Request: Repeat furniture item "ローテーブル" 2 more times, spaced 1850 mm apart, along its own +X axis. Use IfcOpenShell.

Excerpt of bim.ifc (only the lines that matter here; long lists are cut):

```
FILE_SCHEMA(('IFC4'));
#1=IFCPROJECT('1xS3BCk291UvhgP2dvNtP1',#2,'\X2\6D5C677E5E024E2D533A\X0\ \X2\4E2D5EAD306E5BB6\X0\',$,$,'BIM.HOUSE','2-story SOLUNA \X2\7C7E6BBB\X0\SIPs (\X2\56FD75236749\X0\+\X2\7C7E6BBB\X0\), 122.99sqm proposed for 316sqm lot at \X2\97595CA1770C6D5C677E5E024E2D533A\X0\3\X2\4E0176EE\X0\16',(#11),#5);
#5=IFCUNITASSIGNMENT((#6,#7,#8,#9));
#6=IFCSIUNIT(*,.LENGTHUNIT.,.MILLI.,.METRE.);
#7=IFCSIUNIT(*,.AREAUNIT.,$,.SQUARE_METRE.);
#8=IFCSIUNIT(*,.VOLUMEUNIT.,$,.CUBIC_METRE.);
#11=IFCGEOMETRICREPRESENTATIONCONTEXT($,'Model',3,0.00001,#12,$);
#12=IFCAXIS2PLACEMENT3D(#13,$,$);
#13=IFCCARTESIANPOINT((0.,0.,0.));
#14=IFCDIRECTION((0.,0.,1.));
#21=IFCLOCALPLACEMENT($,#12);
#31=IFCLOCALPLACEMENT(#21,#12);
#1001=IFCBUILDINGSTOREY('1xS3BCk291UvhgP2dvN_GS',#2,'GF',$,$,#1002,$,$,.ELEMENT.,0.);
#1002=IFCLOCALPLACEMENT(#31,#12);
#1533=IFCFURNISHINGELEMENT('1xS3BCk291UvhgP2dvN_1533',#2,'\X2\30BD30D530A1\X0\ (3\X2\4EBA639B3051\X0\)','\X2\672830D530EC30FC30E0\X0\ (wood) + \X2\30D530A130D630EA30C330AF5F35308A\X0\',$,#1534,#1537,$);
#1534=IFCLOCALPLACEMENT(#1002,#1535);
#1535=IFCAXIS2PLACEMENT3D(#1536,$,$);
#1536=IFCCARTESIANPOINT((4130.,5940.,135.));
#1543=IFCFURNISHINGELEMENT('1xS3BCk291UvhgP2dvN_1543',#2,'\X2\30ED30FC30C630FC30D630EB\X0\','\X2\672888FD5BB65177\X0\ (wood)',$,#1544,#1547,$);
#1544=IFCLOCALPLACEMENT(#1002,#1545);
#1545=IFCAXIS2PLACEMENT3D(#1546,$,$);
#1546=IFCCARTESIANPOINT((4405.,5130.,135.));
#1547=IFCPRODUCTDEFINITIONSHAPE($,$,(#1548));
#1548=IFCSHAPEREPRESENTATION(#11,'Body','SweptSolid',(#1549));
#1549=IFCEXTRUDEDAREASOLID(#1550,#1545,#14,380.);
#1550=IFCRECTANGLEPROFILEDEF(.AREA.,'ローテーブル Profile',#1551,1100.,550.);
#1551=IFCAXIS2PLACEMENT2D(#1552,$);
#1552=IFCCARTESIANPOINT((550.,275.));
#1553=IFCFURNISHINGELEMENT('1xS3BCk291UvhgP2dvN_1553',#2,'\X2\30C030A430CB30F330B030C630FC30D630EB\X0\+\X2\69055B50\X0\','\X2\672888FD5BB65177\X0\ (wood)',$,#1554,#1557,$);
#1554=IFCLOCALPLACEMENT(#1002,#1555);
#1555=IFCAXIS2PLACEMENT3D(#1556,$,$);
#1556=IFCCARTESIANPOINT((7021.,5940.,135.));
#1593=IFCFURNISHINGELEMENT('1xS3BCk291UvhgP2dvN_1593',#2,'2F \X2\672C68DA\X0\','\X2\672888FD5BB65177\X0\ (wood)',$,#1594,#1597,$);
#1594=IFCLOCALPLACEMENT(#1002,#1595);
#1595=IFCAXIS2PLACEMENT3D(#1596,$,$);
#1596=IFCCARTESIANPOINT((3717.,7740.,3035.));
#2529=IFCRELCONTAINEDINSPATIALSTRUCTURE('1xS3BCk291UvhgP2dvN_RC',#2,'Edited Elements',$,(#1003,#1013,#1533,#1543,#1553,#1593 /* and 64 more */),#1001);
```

```python
import ifcopenshell
import ifcopenshell.api.geometry
import ifcopenshell.api.root
import ifcopenshell.util.element
import ifcopenshell.util.placement

model = ifcopenshell.open("bim.ifc")


def reuse_history(source, copy):
    """copy_class also copies each property set's owner history, people and application; keep the originals."""
    for rel in copy.IsDefinedBy:
        if rel.is_a("IfcRelDefinesByProperties") and (history := rel.RelatingPropertyDefinition.OwnerHistory):
            rel.RelatingPropertyDefinition.OwnerHistory = source.OwnerHistory
            ifcopenshell.util.element.remove_deep2(model, history)


source = model.by_id(1543)
base = ifcopenshell.util.placement.get_local_placement(source.ObjectPlacement)
step = base[:3, 0] * 1850.0

for i in range(1, 3):
    copy = ifcopenshell.api.root.copy_class(model, product=source)
    copy.Representation = ifcopenshell.util.element.copy_deep(
        model, source.Representation, exclude=["IfcGeometricRepresentationContext", "IfcRepresentationMap"]
    )
    reuse_history(source, copy)
    matrix = base.copy()
    matrix[:3, 3] += i * step
    print("added at", matrix[:3, 3].round(3) + 0.0)
    ifcopenshell.api.geometry.edit_object_placement(model, product=copy, matrix=matrix, is_si=False)

model.write("bim_edited.ifc")
```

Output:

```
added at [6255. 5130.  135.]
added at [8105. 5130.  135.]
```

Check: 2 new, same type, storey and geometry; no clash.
